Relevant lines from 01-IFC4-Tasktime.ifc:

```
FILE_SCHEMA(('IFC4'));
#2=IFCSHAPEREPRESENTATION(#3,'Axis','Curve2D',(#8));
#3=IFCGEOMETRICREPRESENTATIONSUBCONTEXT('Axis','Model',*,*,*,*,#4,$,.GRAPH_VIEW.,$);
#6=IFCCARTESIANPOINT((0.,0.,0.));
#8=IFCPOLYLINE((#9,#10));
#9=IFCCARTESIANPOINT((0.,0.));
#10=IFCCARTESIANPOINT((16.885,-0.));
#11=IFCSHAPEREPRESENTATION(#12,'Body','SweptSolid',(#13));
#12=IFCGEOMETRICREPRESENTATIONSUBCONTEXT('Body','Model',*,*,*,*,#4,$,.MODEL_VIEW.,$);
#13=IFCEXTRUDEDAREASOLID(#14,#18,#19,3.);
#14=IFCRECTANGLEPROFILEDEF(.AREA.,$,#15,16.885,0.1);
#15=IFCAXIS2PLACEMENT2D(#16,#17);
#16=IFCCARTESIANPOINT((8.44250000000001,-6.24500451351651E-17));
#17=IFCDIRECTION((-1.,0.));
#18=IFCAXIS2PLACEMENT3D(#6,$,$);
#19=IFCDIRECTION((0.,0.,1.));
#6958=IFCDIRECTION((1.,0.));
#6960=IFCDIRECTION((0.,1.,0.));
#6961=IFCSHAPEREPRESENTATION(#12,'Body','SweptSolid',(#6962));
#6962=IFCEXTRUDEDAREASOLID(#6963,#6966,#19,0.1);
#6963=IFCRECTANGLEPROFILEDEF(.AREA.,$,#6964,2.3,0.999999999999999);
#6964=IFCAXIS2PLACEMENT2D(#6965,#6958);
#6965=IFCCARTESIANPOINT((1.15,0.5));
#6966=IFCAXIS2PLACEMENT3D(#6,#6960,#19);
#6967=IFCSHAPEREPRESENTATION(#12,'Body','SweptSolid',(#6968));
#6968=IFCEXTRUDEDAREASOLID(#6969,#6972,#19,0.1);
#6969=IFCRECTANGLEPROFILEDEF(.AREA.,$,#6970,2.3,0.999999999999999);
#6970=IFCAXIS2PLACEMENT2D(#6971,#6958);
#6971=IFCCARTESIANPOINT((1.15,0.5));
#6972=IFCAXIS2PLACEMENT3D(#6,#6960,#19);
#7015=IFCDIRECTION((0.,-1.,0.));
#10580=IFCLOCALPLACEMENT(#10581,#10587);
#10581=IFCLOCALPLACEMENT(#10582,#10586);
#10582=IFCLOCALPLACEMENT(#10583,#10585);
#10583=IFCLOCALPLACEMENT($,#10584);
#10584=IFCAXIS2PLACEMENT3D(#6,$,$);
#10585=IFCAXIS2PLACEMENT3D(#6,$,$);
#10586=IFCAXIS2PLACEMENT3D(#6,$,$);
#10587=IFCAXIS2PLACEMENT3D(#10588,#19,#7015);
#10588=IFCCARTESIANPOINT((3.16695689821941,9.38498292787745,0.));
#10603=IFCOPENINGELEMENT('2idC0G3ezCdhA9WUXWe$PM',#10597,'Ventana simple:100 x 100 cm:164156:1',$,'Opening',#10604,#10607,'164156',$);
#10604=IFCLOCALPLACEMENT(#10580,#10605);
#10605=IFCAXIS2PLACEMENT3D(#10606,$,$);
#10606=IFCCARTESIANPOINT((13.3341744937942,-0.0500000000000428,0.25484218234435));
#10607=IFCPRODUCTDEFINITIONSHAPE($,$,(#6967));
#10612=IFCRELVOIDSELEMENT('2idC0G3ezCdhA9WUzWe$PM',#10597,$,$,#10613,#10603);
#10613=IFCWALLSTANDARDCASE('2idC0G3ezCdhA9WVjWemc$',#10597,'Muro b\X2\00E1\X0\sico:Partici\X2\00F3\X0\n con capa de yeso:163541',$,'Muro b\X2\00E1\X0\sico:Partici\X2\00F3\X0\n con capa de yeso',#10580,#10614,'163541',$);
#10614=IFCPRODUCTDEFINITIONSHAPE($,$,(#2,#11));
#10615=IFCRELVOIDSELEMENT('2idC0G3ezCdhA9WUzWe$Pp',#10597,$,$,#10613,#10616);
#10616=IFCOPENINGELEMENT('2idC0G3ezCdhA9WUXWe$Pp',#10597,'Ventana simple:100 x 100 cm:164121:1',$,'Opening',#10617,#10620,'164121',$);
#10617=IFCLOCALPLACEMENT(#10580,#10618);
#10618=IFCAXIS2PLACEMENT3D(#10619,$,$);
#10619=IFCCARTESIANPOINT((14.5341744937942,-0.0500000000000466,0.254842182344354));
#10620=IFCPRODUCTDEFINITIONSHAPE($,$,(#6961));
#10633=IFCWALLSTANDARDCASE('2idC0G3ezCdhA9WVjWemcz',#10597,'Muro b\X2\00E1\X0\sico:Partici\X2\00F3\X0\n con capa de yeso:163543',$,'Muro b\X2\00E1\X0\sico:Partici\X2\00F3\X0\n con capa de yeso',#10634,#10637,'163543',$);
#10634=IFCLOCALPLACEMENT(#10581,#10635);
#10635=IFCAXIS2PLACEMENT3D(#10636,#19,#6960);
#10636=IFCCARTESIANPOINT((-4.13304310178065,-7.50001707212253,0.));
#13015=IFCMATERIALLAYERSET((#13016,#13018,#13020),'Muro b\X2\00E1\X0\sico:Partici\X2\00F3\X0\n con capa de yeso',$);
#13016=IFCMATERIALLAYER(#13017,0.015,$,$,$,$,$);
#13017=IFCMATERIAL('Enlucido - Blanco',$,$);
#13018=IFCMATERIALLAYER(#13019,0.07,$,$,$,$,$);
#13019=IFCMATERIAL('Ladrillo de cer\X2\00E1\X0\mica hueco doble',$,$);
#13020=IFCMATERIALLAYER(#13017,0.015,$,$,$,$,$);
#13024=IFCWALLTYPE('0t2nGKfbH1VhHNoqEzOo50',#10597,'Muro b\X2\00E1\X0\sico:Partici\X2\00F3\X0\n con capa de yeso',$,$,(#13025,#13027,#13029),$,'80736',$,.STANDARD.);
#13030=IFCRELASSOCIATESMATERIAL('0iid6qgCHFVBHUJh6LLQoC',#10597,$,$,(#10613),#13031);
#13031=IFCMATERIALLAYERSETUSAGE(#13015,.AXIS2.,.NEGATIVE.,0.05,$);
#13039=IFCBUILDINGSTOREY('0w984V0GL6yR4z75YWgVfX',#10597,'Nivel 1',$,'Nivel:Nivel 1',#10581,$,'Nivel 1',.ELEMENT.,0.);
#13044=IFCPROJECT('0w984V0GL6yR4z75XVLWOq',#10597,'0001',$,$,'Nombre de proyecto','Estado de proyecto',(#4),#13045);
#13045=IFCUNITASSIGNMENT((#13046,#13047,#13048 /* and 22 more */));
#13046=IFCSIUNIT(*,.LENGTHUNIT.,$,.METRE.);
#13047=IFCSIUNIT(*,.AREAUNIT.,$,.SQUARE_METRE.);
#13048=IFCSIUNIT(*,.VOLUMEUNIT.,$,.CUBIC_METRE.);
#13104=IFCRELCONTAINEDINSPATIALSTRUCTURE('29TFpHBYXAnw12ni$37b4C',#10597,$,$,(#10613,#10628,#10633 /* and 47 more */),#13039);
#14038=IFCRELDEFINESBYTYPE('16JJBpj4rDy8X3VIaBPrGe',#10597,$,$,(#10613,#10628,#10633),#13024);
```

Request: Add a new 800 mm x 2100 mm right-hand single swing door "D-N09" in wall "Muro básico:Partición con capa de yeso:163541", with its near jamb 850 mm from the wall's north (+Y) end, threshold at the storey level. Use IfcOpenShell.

```python
import numpy as np
import ifcopenshell
import ifcopenshell.api.feature
import ifcopenshell.api.geometry
import ifcopenshell.api.root
import ifcopenshell.api.spatial
import ifcopenshell.geom
import ifcopenshell.util.element
import ifcopenshell.util.placement
import ifcopenshell.util.representation
import ifcopenshell.util.shape
import ifcopenshell.util.unit

model = ifcopenshell.open("01-IFC4-Tasktime.ifc")
unit_scale = ifcopenshell.util.unit.calculate_unit_scale(model)
settings = ifcopenshell.geom.settings()


def volume(element):
    """Net volume in cubic metres, openings subtracted."""
    shape = ifcopenshell.geom.create_shape(settings, element)
    return ifcopenshell.util.shape.get_volume(shape.geometry)


wall = model.by_guid("2idC0G3ezCdhA9WVjWemc$")
storey = ifcopenshell.util.element.get_container(wall, ifc_class="IfcBuildingStorey")
context = ifcopenshell.util.representation.get_context(model, "Model", "Body", "MODEL_VIEW")
before = volume(wall)

width, height, from_end, sill = 0.8, 2.1, 0.85, 0.0  # metres

# The wall runs along its own X axis, and the end named is its -X end.
wall_shape = ifcopenshell.geom.create_shape(settings, wall)
x, y, z = ifcopenshell.util.shape.get_vertices(wall_shape.geometry).T
start = x.min() + from_end
face, thickness = float(y.min()), float(y.max() - y.min())
wall_matrix = ifcopenshell.util.placement.get_local_placement(wall.ObjectPlacement)
level = ifcopenshell.util.placement.get_local_placement(storey.ObjectPlacement)[2, 3]


def in_wall(x, y):
    """Placement at x, y metres in the wall's axes, at sill height."""
    matrix = wall_matrix.copy()
    matrix[:, 3] = wall_matrix @ np.array([x / unit_scale, y / unit_scale, 0.0, 1.0])
    matrix[2, 3] = level + sill / unit_scale
    return matrix


# Opening: a box that overshoots both wall faces by 50 mm.
opening = ifcopenshell.api.root.create_entity(model, ifc_class="IfcOpeningElement", predefined_type="OPENING")
box = ifcopenshell.api.geometry.add_wall_representation(
    model, context=context, length=width, height=height, thickness=thickness + 0.1
)
ifcopenshell.api.geometry.assign_representation(model, product=opening, representation=box)
ifcopenshell.api.geometry.edit_object_placement(model, product=opening, matrix=in_wall(start, face - 0.05), is_si=False)
ifcopenshell.api.feature.add_feature(model, feature=opening, element=wall)

door = ifcopenshell.api.root.create_entity(model, ifc_class="IfcDoor", name="D-N09", predefined_type="DOOR")
door.OverallWidth, door.OverallHeight = width / unit_scale, height / unit_scale
door.OperationType = "SINGLE_SWING_RIGHT"
body = ifcopenshell.api.geometry.add_door_representation(
    model,
    context=context,
    overall_width=door.OverallWidth,
    overall_height=door.OverallHeight,
    operation_type="SINGLE_SWING_RIGHT",
    lining_properties={"LiningDepth": thickness / unit_scale, "ThresholdDepth": thickness / unit_scale},
)
ifcopenshell.api.geometry.assign_representation(model, product=door, representation=body)
ifcopenshell.api.spatial.assign_container(model, products=[door], relating_structure=storey)
ifcopenshell.api.feature.add_filling(model, opening=opening, element=door)

# The lining spans the wall, so the door starts at the wall face.
ifcopenshell.api.geometry.edit_object_placement(model, product=door, matrix=in_wall(start, face), is_si=False)

after = volume(wall)

print(f"wall volume {before:.3f} -> {after:.3f} m3")

model.write("01-IFC4-Tasktime_edited.ifc")
```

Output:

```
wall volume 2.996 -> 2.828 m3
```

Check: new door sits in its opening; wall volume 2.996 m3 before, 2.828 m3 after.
